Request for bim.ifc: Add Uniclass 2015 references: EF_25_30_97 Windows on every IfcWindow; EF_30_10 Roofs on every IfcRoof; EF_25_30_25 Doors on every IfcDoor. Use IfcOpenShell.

First a look at what the model holds.

```python
import ifcopenshell

model = ifcopenshell.open("bim.ifc")
print(model.schema)
print("classifications:", [c.Name for c in model.by_type("IfcClassification")])
for ifc_class in ("IfcDoor", "IfcRoof", "IfcStair", "IfcWall", "IfcWindow"):
    print(ifc_class, len(model.by_type(ifc_class)))
```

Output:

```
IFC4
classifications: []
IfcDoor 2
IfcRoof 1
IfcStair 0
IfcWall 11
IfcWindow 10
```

```python
import ifcopenshell
import ifcopenshell.api.classification

model = ifcopenshell.open("bim.ifc")

system = ifcopenshell.api.classification.add_classification(model, classification="Uniclass 2015")

codes = {
    "IfcWindow": ("EF_25_30_97", "Windows"),
    "IfcRoof": ("EF_30_10", "Roofs"),
    "IfcDoor": ("EF_25_30_25", "Doors"),
}
for ifc_class, (code, name) in codes.items():
    products = model.by_type(ifc_class)
    ifcopenshell.api.classification.add_reference(
        model, products=products, classification=system, identification=code, name=name
    )
    print(code, len(products))

model.write("bim_updated.ifc")
```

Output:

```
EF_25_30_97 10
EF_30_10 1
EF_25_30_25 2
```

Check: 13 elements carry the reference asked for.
